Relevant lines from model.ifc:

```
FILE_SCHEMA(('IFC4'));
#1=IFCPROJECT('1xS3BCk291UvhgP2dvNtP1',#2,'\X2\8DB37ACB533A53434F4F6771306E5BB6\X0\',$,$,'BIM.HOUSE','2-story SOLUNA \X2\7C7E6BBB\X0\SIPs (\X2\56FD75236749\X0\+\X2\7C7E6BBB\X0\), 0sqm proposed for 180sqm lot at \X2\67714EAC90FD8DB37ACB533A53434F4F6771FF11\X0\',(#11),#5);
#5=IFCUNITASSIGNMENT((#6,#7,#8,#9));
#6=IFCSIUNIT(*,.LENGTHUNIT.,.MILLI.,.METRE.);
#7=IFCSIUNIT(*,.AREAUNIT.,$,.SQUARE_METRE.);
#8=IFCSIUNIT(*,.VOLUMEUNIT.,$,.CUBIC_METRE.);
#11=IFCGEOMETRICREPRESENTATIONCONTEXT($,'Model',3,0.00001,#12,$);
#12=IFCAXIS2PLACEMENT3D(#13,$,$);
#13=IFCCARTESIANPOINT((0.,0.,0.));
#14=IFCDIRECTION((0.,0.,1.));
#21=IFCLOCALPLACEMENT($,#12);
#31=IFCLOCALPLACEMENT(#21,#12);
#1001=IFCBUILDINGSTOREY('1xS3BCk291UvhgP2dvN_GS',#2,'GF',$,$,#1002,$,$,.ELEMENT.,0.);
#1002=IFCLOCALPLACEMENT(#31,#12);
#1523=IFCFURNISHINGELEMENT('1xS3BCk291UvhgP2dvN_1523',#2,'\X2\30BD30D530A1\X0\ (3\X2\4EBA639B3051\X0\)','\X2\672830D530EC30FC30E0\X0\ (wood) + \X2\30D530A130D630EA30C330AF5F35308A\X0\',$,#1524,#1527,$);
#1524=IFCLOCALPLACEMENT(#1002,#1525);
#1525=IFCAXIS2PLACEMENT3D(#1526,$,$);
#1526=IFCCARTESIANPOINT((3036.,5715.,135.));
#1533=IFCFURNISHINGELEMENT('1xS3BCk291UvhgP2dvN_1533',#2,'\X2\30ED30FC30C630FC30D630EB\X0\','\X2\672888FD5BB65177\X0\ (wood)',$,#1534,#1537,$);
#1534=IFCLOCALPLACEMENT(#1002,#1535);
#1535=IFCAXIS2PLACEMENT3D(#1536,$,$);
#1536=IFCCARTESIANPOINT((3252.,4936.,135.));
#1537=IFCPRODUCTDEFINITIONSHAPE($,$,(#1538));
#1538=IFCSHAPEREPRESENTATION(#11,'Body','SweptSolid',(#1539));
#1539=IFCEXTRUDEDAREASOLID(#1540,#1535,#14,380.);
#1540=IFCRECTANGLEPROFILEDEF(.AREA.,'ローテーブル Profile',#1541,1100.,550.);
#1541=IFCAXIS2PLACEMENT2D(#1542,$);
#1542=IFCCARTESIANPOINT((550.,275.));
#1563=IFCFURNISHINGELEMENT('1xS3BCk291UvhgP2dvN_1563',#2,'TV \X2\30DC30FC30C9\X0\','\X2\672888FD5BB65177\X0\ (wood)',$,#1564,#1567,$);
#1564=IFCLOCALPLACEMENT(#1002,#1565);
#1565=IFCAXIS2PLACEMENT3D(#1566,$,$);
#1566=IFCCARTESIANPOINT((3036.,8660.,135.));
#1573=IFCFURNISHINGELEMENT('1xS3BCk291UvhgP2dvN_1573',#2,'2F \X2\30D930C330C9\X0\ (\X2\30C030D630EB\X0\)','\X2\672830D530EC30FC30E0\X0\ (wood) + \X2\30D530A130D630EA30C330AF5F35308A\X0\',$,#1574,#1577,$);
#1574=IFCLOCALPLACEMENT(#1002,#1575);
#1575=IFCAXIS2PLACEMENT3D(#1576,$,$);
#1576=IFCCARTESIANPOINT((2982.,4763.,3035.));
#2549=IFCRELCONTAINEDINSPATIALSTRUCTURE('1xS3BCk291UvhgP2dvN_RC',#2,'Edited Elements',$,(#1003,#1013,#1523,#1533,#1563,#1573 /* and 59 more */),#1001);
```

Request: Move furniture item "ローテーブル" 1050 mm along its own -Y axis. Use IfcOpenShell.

```python
import ifcopenshell
import ifcopenshell.api.geometry
import ifcopenshell.util.placement
import ifcopenshell.util.unit

model = ifcopenshell.open("model.ifc")
unit_scale = ifcopenshell.util.unit.calculate_unit_scale(model)

item = model.by_id(1533)
matrix = ifcopenshell.util.placement.get_local_placement(item.ObjectPlacement)
matrix[:3, 3] -= matrix[:3, 1] * 1.05 / unit_scale
ifcopenshell.api.geometry.edit_object_placement(model, product=item, matrix=matrix, is_si=False)

print(ifcopenshell.util.placement.get_local_placement(item.ObjectPlacement).round(3) + 0.0)

model.write("model_rev.ifc")
```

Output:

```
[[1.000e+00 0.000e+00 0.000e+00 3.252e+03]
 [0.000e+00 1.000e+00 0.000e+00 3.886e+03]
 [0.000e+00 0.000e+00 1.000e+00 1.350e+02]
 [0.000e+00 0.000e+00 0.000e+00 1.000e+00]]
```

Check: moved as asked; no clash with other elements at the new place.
